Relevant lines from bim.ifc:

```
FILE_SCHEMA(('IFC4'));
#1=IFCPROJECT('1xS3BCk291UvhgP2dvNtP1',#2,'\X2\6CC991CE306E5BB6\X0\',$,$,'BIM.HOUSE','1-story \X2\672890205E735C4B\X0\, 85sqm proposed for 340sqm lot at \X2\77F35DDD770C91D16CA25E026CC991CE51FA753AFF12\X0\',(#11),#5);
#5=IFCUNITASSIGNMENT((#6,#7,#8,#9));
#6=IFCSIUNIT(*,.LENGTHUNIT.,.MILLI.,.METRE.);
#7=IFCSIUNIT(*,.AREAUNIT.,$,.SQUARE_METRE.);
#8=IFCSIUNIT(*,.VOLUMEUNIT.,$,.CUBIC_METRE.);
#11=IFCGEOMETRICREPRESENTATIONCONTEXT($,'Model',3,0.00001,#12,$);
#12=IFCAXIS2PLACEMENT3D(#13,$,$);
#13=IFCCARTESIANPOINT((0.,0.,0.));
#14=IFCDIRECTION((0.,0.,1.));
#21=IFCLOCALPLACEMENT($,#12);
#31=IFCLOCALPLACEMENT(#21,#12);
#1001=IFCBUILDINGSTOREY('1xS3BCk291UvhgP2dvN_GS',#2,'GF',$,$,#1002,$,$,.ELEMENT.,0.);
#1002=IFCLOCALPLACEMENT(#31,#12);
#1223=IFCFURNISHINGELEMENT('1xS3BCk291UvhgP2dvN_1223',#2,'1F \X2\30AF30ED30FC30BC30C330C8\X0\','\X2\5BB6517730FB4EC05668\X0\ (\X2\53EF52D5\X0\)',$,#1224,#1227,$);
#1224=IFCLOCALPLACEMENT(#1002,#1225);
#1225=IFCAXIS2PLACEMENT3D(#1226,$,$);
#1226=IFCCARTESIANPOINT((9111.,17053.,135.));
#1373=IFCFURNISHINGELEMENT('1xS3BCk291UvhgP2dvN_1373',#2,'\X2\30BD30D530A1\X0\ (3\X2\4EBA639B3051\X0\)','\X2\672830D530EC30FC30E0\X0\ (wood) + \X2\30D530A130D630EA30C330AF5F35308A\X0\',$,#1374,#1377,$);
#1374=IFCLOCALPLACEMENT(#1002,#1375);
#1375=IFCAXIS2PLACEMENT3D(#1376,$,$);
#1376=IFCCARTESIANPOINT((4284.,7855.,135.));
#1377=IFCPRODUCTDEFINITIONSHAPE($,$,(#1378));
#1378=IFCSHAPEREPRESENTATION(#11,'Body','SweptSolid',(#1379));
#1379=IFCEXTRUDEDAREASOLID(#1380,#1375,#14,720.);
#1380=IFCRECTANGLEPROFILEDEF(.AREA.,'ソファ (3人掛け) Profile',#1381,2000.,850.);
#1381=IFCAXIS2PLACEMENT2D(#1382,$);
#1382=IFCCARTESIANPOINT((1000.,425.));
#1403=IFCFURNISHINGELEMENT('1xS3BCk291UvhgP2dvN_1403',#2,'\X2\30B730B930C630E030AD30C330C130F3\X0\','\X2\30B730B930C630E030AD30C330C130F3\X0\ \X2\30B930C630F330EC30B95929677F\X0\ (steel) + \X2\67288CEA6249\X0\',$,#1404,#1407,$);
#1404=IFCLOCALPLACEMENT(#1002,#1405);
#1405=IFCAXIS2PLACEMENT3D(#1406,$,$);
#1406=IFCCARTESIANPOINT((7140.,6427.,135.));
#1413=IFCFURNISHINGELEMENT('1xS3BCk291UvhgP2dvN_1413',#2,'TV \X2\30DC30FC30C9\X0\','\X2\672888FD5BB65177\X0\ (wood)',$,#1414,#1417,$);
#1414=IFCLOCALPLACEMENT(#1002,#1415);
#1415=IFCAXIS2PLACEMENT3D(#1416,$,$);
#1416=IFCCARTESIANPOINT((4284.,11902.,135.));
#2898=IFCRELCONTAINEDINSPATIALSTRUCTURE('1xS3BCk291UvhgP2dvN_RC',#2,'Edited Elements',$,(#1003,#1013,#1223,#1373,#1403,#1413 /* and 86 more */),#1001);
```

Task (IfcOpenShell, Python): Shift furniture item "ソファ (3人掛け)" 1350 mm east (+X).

```python
import ifcopenshell
import ifcopenshell.api.geometry
import ifcopenshell.util.placement
import ifcopenshell.util.unit

model = ifcopenshell.open("bim.ifc")
unit_scale = ifcopenshell.util.unit.calculate_unit_scale(model)

item = model.by_guid("1xS3BCk291UvhgP2dvN_1373")
matrix = ifcopenshell.util.placement.get_local_placement(item.ObjectPlacement)
matrix[0, 3] += 1.35 / unit_scale
ifcopenshell.api.geometry.edit_object_placement(model, product=item, matrix=matrix, is_si=False)

print(ifcopenshell.util.placement.get_local_placement(item.ObjectPlacement).round(3) + 0.0)

model.write("bim_updated.ifc")
```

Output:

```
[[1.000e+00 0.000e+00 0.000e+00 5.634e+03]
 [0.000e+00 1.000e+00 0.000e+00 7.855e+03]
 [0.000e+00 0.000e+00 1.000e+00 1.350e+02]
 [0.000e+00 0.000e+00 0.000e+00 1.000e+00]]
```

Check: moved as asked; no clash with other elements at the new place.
